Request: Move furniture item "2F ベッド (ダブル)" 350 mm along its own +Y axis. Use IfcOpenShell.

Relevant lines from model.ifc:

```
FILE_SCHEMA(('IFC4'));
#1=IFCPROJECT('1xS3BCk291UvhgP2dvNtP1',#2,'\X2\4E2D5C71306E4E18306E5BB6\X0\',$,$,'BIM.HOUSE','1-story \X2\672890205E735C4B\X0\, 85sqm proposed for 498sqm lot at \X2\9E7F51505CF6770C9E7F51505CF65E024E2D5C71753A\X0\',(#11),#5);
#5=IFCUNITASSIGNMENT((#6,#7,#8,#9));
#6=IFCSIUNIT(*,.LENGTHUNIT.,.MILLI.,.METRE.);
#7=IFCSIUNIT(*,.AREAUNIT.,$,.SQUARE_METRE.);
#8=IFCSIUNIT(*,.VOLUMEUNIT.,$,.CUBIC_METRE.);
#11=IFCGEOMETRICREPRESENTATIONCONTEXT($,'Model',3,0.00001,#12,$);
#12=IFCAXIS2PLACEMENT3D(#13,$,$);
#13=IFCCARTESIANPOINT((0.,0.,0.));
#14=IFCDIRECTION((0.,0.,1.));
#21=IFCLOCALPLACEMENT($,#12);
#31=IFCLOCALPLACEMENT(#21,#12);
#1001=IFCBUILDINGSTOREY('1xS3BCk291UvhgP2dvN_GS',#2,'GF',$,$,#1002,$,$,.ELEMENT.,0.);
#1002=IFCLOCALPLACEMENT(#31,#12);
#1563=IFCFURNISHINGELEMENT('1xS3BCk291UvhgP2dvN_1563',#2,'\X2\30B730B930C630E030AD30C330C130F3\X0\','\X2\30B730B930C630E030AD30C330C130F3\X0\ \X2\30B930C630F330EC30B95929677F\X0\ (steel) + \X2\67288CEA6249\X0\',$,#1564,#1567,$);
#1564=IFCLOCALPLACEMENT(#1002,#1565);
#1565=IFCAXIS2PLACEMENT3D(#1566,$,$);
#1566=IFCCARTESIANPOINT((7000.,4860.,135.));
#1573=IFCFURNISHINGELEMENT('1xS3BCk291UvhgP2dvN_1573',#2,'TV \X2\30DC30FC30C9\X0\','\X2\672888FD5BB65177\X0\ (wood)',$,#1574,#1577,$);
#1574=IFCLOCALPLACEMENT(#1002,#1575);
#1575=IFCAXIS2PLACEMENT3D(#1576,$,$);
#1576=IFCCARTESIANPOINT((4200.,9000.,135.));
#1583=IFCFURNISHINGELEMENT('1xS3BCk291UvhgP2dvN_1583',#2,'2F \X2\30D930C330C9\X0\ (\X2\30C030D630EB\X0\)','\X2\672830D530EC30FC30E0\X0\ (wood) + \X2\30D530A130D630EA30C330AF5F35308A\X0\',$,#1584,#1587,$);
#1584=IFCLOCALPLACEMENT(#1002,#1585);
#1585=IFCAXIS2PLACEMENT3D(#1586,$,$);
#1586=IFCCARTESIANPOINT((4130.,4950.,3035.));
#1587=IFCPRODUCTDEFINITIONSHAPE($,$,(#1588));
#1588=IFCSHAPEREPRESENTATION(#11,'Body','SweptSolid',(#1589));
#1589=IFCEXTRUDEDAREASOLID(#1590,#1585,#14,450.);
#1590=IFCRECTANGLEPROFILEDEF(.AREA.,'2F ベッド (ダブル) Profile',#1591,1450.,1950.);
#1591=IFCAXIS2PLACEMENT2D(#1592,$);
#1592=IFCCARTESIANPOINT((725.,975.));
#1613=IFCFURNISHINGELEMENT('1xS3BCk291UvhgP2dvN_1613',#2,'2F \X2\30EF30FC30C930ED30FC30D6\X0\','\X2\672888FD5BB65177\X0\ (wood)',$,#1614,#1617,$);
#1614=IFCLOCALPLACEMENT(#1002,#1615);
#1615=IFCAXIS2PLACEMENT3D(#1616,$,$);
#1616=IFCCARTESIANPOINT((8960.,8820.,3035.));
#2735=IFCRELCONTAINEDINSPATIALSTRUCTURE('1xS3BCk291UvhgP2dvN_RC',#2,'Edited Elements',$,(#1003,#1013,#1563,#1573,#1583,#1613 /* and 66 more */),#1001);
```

```python
import ifcopenshell
import ifcopenshell.api.geometry
import ifcopenshell.util.placement

model = ifcopenshell.open("model.ifc")

item = model.by_guid("1xS3BCk291UvhgP2dvN_1583")
matrix = ifcopenshell.util.placement.get_local_placement(item.ObjectPlacement)
matrix[:3, 3] += matrix[:3, 1] * 350.0
ifcopenshell.api.geometry.edit_object_placement(model, product=item, matrix=matrix, is_si=False)

print(ifcopenshell.util.placement.get_local_placement(item.ObjectPlacement).round(3) + 0.0)

model.write("model_updated.ifc")
```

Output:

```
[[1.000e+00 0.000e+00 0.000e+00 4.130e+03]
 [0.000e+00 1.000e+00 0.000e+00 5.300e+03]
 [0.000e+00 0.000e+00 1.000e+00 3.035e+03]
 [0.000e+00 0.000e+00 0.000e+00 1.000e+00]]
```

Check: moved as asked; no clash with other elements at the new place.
